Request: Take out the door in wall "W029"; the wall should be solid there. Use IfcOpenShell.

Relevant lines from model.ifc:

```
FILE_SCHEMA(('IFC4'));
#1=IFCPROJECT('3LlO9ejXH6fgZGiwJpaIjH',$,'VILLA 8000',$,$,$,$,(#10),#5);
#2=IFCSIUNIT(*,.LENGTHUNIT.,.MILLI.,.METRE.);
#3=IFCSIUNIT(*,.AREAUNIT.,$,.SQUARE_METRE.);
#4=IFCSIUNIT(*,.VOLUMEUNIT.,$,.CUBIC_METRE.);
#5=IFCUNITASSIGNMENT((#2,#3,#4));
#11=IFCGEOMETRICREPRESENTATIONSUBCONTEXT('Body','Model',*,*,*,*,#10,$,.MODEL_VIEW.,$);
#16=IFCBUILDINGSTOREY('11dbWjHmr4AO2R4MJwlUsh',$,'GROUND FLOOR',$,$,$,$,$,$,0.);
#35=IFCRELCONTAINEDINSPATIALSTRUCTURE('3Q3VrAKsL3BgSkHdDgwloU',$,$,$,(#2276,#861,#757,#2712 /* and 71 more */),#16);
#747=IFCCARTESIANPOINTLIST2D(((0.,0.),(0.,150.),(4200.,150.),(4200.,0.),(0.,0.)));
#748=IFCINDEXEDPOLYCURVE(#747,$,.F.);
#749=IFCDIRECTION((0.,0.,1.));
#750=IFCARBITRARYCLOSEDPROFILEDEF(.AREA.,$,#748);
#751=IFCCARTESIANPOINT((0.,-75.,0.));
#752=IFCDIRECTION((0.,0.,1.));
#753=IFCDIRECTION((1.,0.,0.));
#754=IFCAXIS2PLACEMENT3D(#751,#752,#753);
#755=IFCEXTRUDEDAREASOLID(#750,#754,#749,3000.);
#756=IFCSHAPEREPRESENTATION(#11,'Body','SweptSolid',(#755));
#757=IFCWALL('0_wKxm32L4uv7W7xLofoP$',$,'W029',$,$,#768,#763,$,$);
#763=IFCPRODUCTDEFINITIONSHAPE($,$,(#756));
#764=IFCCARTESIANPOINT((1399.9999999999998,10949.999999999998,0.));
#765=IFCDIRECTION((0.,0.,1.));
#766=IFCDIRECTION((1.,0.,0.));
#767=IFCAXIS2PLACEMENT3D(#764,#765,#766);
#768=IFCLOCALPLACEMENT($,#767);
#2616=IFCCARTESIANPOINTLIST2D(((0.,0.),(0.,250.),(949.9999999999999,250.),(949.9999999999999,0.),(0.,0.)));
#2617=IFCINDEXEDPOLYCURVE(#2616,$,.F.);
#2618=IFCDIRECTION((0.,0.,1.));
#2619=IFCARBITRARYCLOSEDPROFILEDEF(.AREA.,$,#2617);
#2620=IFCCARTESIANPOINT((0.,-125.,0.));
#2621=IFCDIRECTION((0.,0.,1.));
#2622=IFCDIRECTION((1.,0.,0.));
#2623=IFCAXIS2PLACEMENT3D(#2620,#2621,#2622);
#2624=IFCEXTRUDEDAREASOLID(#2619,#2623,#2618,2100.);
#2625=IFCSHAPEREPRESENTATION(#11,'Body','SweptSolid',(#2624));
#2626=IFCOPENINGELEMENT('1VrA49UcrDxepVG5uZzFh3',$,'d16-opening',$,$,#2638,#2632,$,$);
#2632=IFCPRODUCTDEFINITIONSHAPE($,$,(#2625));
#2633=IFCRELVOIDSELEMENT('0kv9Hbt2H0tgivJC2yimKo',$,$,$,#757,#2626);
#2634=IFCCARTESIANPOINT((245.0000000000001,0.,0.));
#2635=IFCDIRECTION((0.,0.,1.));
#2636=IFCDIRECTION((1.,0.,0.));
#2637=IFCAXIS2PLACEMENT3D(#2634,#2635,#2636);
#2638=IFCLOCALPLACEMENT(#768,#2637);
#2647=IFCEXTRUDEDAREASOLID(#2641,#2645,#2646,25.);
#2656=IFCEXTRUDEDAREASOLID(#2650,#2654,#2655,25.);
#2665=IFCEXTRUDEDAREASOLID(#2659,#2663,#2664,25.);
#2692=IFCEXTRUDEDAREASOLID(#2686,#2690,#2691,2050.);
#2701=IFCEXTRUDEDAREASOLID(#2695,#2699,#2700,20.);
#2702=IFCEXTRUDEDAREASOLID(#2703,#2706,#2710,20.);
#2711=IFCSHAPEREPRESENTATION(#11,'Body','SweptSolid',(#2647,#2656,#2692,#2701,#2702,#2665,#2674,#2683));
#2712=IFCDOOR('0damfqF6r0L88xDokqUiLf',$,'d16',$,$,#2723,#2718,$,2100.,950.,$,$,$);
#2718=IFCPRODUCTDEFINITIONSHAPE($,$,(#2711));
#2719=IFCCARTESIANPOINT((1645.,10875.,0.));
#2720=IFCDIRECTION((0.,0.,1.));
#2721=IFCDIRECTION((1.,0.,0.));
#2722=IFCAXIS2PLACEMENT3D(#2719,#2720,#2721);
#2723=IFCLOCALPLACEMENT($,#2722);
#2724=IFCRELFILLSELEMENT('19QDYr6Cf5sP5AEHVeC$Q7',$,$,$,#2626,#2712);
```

```python
import ifcopenshell
import ifcopenshell.api.feature
import ifcopenshell.api.root
import ifcopenshell.geom
import ifcopenshell.util.shape

model = ifcopenshell.open("model.ifc")
settings = ifcopenshell.geom.settings()


def volume(element):
    """Net volume in cubic metres, openings subtracted."""
    shape = ifcopenshell.geom.create_shape(settings, element)
    return ifcopenshell.util.shape.get_volume(shape.geometry)


door = model.by_guid("0damfqF6r0L88xDokqUiLf")
opening = door.FillsVoids[0].RelatingOpeningElement
wall = opening.VoidsElements[0].RelatingBuildingElement
before = volume(wall)

ifcopenshell.api.root.remove_product(model, product=door)
ifcopenshell.api.feature.remove_feature(model, feature=opening)

after = volume(wall)

print(f"wall volume {before:.3f} -> {after:.3f} m3")

model.write("model_updated.ifc")
```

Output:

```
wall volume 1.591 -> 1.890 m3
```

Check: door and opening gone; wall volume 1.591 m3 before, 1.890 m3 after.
